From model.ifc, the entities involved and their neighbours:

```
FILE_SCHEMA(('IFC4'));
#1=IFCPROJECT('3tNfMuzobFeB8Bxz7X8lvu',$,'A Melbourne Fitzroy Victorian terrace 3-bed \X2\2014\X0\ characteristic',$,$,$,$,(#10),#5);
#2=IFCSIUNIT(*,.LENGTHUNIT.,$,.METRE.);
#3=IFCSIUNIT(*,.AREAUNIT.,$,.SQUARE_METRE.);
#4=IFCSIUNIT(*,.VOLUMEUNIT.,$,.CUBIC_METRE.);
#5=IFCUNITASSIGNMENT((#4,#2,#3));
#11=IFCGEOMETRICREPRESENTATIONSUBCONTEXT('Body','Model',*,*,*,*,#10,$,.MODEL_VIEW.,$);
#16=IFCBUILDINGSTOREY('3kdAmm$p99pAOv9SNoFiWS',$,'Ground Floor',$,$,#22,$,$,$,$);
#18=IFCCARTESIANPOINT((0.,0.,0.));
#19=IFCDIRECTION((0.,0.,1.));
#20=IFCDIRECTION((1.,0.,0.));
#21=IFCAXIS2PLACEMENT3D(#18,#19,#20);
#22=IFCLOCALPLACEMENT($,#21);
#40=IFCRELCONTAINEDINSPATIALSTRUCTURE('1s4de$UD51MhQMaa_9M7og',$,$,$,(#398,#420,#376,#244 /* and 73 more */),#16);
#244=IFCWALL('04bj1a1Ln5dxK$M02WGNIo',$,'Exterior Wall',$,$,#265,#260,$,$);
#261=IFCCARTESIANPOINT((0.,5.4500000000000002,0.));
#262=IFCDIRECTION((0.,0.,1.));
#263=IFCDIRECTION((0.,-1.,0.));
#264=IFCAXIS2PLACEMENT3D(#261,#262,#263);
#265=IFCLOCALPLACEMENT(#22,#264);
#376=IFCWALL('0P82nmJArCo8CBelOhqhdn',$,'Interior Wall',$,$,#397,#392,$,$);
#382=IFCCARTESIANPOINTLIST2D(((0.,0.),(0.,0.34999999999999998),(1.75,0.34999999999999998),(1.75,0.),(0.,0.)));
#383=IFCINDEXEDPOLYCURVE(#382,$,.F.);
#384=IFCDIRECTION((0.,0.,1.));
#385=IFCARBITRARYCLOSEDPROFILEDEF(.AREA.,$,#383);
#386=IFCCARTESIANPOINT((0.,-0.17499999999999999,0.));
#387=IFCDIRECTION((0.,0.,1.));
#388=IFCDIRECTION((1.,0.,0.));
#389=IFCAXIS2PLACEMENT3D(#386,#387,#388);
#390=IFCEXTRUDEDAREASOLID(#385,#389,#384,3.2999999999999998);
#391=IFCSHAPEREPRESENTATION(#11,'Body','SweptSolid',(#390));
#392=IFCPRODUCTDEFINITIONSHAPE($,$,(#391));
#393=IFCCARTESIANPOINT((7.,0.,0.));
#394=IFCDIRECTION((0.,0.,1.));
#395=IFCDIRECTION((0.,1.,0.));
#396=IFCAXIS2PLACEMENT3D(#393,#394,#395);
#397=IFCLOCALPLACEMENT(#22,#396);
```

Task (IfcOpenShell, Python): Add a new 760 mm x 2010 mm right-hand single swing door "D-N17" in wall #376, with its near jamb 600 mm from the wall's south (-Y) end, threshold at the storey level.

```python
import numpy as np
import ifcopenshell
import ifcopenshell.api.feature
import ifcopenshell.api.geometry
import ifcopenshell.api.root
import ifcopenshell.api.spatial
import ifcopenshell.geom
import ifcopenshell.util.element
import ifcopenshell.util.placement
import ifcopenshell.util.representation
import ifcopenshell.util.shape
import ifcopenshell.util.unit

model = ifcopenshell.open("model.ifc")
unit_scale = ifcopenshell.util.unit.calculate_unit_scale(model)
settings = ifcopenshell.geom.settings()


def volume(element):
    """Net volume in cubic metres, openings subtracted."""
    shape = ifcopenshell.geom.create_shape(settings, element)
    return ifcopenshell.util.shape.get_volume(shape.geometry)


wall = model.by_id(376)
storey = ifcopenshell.util.element.get_container(wall, ifc_class="IfcBuildingStorey")
context = ifcopenshell.util.representation.get_context(model, "Model", "Body", "MODEL_VIEW")
before = volume(wall)

width, height, from_end, sill = 0.76, 2.01, 0.6, 0.0  # metres

# The wall runs along its own X axis, and the end named is its -X end.
wall_shape = ifcopenshell.geom.create_shape(settings, wall)
x, y, z = ifcopenshell.util.shape.get_vertices(wall_shape.geometry).T
start = x.min() + from_end
face, thickness = float(y.min()), float(y.max() - y.min())
wall_matrix = ifcopenshell.util.placement.get_local_placement(wall.ObjectPlacement)
level = ifcopenshell.util.placement.get_local_placement(storey.ObjectPlacement)[2, 3]


def in_wall(x, y):
    """Placement at x, y metres in the wall's axes, at sill height."""
    matrix = wall_matrix.copy()
    matrix[:, 3] = wall_matrix @ np.array([x / unit_scale, y / unit_scale, 0.0, 1.0])
    matrix[2, 3] = level + sill / unit_scale
    return matrix


# Opening: a box that overshoots both wall faces by 50 mm.
opening = ifcopenshell.api.root.create_entity(model, ifc_class="IfcOpeningElement", predefined_type="OPENING")
box = ifcopenshell.api.geometry.add_wall_representation(
    model, context=context, length=width, height=height, thickness=thickness + 0.1
)
ifcopenshell.api.geometry.assign_representation(model, product=opening, representation=box)
ifcopenshell.api.geometry.edit_object_placement(model, product=opening, matrix=in_wall(start, face - 0.05), is_si=False)
ifcopenshell.api.feature.add_feature(model, feature=opening, element=wall)

door = ifcopenshell.api.root.create_entity(model, ifc_class="IfcDoor", name="D-N17", predefined_type="DOOR")
door.OverallWidth, door.OverallHeight = width / unit_scale, height / unit_scale
door.OperationType = "SINGLE_SWING_RIGHT"
body = ifcopenshell.api.geometry.add_door_representation(
    model,
    context=context,
    overall_width=door.OverallWidth,
    overall_height=door.OverallHeight,
    operation_type="SINGLE_SWING_RIGHT",
    lining_properties={"LiningDepth": thickness / unit_scale, "ThresholdDepth": thickness / unit_scale},
)
ifcopenshell.api.geometry.assign_representation(model, product=door, representation=body)
ifcopenshell.api.spatial.assign_container(model, products=[door], relating_structure=storey)
ifcopenshell.api.feature.add_filling(model, opening=opening, element=door)

# The lining spans the wall, so the door starts at the wall face.
ifcopenshell.api.geometry.edit_object_placement(model, product=door, matrix=in_wall(start, face), is_si=False)

after = volume(wall)

print(f"wall volume {before:.3f} -> {after:.3f} m3")

model.write("model_v2.ifc")
```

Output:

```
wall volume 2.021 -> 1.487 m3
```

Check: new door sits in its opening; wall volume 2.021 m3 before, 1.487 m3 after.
